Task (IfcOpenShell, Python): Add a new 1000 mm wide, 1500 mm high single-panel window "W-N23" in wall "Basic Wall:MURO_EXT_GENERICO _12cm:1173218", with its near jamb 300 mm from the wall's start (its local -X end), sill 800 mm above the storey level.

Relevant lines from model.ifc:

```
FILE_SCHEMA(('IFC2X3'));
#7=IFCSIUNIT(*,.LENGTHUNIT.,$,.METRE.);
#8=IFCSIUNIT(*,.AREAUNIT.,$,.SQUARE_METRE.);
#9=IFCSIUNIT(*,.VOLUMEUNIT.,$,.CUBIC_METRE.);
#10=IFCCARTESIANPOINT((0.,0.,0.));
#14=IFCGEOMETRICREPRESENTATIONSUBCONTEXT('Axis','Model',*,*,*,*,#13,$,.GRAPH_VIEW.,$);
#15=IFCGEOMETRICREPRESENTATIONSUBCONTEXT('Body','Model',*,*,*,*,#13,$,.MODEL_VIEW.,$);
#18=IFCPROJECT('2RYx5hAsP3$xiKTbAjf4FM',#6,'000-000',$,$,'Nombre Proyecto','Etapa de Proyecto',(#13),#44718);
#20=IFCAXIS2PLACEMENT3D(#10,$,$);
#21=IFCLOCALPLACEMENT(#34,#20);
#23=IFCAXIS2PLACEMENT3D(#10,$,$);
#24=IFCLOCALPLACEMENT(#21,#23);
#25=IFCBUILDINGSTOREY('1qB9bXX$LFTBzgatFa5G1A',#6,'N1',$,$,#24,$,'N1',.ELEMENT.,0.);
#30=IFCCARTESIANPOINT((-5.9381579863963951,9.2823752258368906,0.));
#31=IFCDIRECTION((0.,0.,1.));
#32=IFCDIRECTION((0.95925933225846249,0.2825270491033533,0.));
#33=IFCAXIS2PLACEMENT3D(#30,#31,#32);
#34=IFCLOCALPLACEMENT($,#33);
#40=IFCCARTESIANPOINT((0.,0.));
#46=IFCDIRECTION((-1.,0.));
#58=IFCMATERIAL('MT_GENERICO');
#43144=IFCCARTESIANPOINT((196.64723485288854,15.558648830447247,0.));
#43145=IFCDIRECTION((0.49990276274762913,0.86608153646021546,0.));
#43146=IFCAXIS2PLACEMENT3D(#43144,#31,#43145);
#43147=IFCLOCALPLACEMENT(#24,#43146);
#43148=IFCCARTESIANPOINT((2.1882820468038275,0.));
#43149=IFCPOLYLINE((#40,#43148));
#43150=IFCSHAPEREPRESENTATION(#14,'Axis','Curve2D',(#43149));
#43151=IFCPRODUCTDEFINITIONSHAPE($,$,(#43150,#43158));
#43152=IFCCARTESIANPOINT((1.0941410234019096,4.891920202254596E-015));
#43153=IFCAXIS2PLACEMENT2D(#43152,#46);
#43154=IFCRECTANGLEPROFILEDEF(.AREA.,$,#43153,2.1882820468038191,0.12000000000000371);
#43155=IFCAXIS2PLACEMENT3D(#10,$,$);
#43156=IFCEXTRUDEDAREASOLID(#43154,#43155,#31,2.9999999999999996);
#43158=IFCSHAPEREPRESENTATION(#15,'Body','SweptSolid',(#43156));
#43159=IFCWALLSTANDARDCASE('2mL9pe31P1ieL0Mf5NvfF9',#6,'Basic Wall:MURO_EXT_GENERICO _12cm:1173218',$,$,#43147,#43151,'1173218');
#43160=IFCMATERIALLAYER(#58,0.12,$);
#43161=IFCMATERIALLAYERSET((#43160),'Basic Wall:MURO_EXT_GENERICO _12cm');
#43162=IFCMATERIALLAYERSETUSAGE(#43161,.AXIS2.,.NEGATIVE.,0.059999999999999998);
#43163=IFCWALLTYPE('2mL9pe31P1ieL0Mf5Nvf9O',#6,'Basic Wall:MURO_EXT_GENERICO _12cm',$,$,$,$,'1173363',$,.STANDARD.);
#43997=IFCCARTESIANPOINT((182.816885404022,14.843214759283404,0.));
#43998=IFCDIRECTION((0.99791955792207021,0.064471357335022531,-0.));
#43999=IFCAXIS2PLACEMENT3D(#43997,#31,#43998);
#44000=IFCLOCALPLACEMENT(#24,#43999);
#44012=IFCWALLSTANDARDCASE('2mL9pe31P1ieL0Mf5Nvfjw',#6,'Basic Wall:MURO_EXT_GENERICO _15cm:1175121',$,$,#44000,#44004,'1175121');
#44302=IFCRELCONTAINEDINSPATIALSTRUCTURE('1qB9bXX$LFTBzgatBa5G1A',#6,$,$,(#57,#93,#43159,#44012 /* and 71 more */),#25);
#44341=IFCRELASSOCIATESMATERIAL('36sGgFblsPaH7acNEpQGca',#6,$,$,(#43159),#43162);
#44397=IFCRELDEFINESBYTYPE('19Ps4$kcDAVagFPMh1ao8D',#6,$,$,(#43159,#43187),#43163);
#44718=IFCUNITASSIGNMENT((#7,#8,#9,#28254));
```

```python
import numpy as np
import ifcopenshell
import ifcopenshell.api.feature
import ifcopenshell.api.geometry
import ifcopenshell.api.root
import ifcopenshell.api.spatial
import ifcopenshell.api.type
import ifcopenshell.geom
import ifcopenshell.util.element
import ifcopenshell.util.placement
import ifcopenshell.util.representation
import ifcopenshell.util.shape
import ifcopenshell.util.unit

model = ifcopenshell.open("model.ifc")
unit_scale = ifcopenshell.util.unit.calculate_unit_scale(model)
settings = ifcopenshell.geom.settings()


def volume(element):
    """Net volume in cubic metres, openings subtracted."""
    shape = ifcopenshell.geom.create_shape(settings, element)
    return ifcopenshell.util.shape.get_volume(shape.geometry)


wall = model.by_guid("2mL9pe31P1ieL0Mf5NvfF9")
storey = ifcopenshell.util.element.get_container(wall, ifc_class="IfcBuildingStorey")
context = ifcopenshell.util.representation.get_context(model, "Model", "Body", "MODEL_VIEW")
before = volume(wall)

width, height, from_end, sill = 1, 1.5, 0.3, 0.8  # metres

# The wall runs along its own X axis, and the end named is its -X end.
wall_shape = ifcopenshell.geom.create_shape(settings, wall)
x, y, z = ifcopenshell.util.shape.get_vertices(wall_shape.geometry).T
start = x.min() + from_end
face, thickness = float(y.min()), float(y.max() - y.min())
wall_matrix = ifcopenshell.util.placement.get_local_placement(wall.ObjectPlacement)
level = ifcopenshell.util.placement.get_local_placement(storey.ObjectPlacement)[2, 3]


def in_wall(x, y):
    """Placement at x, y metres in the wall's axes, at sill height."""
    matrix = wall_matrix.copy()
    matrix[:, 3] = wall_matrix @ np.array([x / unit_scale, y / unit_scale, 0.0, 1.0])
    matrix[2, 3] = level + sill / unit_scale
    return matrix


# Opening: a box that overshoots both wall faces by 50 mm.
opening = ifcopenshell.api.root.create_entity(model, ifc_class="IfcOpeningElement")
box = ifcopenshell.api.geometry.add_wall_representation(
    model, context=context, length=width, height=height, thickness=thickness + 0.1
)
ifcopenshell.api.geometry.assign_representation(model, product=opening, representation=box)
ifcopenshell.api.geometry.edit_object_placement(model, product=opening, matrix=in_wall(start, face - 0.05), is_si=False)
ifcopenshell.api.feature.add_feature(model, feature=opening, element=wall)

window = ifcopenshell.api.root.create_entity(model, ifc_class="IfcWindow", name="W-N23")
window.OverallWidth, window.OverallHeight = width / unit_scale, height / unit_scale
body = ifcopenshell.api.geometry.add_window_representation(
    model,
    context=context,
    overall_width=window.OverallWidth,
    overall_height=window.OverallHeight,
    partition_type="SINGLE_PANEL",
)
ifcopenshell.api.geometry.assign_representation(model, product=window, representation=body)
ifcopenshell.api.spatial.assign_container(model, products=[window], relating_structure=storey)
fills = ifcopenshell.api.feature.add_filling(model, opening=opening, element=window)
fills.OwnerHistory = window.OwnerHistory  # required in IFC2X3

# IFC2X3 keeps the operation on the window style.
style = ifcopenshell.api.root.create_entity(model, ifc_class="IfcWindowStyle", name="W-N23")
style.OperationType, style.ConstructionType = "SINGLE_PANEL", "NOTDEFINED"
style.ParameterTakesPrecedence = style.Sizeable = False
ifcopenshell.api.type.assign_type(model, related_objects=[window], relating_type=style)

# Centre the window in the wall's thickness.
ifcopenshell.api.geometry.edit_object_placement(model, product=window, matrix=in_wall(start, face), is_si=False)
window_shape = ifcopenshell.geom.create_shape(settings, window)
depth = ifcopenshell.util.shape.get_vertices(window_shape.geometry)[:, 1]
offset = face + thickness / 2 - (depth.min() + depth.max()) / 2
ifcopenshell.api.geometry.edit_object_placement(model, product=window, matrix=in_wall(start, offset), is_si=False)

after = volume(wall)

print(f"wall volume {before:.3f} -> {after:.3f} m3")

model.write("model_v2.ifc")
```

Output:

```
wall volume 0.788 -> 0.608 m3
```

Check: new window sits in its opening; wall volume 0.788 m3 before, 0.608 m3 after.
